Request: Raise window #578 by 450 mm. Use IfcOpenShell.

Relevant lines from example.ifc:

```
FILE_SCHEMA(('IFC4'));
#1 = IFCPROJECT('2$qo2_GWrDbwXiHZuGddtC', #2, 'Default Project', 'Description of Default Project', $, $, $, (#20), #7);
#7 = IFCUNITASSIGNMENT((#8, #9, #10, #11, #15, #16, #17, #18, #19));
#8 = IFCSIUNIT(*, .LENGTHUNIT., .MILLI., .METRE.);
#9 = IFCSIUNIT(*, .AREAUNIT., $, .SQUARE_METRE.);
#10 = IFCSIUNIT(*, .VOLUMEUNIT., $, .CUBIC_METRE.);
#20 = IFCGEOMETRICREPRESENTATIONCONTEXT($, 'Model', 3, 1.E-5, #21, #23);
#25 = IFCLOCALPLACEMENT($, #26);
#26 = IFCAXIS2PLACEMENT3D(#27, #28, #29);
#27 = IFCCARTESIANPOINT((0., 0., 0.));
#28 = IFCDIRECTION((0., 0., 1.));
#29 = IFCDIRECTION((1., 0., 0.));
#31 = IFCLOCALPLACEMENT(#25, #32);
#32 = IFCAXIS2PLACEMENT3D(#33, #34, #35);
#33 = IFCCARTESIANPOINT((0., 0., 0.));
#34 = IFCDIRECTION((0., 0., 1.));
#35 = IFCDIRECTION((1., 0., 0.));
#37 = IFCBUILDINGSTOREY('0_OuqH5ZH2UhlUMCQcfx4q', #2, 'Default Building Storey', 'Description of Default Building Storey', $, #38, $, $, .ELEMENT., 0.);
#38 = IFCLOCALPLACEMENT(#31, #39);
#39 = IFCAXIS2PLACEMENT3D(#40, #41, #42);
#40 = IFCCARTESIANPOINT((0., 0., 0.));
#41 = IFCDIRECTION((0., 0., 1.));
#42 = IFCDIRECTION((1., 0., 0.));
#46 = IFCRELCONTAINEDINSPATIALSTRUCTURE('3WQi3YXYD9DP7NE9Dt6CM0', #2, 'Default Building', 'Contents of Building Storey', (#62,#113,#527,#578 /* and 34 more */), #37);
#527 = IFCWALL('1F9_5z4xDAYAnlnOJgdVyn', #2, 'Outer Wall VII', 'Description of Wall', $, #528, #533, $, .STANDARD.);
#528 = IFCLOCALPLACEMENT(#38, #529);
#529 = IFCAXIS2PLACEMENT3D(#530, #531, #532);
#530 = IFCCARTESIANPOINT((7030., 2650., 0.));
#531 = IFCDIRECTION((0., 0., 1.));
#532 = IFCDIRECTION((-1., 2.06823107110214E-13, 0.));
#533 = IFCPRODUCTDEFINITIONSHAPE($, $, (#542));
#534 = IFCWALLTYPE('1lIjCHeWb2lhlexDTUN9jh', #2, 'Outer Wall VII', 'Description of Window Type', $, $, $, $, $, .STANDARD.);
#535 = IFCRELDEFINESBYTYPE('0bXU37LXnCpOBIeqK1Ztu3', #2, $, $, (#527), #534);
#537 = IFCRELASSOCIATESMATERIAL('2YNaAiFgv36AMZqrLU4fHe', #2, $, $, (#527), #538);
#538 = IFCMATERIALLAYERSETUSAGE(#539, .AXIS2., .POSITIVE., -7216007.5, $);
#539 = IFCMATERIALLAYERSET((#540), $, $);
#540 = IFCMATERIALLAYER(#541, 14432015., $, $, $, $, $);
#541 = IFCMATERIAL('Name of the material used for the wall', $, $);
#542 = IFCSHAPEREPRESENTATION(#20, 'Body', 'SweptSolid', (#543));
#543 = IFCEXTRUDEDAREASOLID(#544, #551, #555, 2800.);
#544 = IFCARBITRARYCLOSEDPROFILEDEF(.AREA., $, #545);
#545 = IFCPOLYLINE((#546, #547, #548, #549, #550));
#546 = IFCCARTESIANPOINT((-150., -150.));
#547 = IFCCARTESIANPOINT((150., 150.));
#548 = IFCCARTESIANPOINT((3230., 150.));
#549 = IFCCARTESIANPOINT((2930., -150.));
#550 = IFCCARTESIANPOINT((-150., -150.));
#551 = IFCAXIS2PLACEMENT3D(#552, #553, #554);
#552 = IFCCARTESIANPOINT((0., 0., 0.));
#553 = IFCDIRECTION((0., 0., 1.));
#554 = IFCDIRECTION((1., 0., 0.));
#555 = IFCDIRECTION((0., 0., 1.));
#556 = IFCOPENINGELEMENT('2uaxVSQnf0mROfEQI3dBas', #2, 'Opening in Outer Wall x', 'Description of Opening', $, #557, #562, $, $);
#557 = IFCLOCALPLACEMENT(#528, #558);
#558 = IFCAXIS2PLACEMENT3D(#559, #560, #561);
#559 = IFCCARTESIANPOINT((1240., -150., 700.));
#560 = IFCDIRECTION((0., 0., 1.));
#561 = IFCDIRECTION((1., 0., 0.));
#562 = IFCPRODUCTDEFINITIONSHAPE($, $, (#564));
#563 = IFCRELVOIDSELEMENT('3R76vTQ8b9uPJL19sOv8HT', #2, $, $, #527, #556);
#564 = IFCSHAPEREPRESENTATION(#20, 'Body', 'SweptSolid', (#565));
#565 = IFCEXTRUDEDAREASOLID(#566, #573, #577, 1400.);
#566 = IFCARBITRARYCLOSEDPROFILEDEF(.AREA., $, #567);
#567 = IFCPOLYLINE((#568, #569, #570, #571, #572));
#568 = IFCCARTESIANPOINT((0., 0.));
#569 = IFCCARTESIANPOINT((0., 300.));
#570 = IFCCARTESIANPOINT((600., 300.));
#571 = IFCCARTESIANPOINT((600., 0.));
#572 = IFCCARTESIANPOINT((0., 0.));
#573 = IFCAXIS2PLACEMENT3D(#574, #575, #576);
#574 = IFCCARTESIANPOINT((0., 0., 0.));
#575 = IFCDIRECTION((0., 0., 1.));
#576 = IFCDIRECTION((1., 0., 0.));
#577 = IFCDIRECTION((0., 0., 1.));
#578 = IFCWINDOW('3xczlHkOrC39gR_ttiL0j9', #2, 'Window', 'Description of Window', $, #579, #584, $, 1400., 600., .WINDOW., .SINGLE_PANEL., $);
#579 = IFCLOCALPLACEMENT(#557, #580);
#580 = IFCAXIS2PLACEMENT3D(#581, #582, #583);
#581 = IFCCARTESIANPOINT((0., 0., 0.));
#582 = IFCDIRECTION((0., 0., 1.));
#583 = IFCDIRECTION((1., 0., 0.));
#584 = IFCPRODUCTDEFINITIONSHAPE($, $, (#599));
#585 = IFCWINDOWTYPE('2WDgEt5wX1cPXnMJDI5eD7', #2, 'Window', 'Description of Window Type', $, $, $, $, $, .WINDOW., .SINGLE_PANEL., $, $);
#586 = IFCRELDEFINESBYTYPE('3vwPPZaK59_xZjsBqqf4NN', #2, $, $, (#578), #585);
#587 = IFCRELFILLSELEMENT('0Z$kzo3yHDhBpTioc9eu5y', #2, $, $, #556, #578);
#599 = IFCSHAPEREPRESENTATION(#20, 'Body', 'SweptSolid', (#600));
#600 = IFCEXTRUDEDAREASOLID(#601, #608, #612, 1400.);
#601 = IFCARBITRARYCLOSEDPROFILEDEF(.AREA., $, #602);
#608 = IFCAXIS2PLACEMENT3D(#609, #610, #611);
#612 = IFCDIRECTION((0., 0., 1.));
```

```python
import numpy as np
import ifcopenshell
import ifcopenshell.api.geometry
import ifcopenshell.util.placement
import ifcopenshell.util.unit

model = ifcopenshell.open("example.ifc")
unit_scale = ifcopenshell.util.unit.calculate_unit_scale(model)

window = model.by_guid("3xczlHkOrC39gR_ttiL0j9")
opening = window.FillsVoids[0].RelatingOpeningElement
dz = 0.45 / unit_scale

shift = np.array([0.0, 0.0, dz])
# The window is placed relative to its opening, so it follows when the opening moves.
matrix = ifcopenshell.util.placement.get_local_placement(opening.ObjectPlacement)
matrix[:3, 3] += shift
ifcopenshell.api.geometry.edit_object_placement(
    model, product=opening, matrix=matrix, is_si=False, should_transform_children=True
)

print(f"moved by {dz * unit_scale:+.3f} m")

model.write("example_edited.ifc")
```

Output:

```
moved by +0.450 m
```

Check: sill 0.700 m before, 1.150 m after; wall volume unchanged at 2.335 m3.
